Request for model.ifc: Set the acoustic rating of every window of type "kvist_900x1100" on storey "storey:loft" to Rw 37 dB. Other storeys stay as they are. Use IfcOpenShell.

First a look at what the model holds.

```python
import ifcopenshell
import ifcopenshell.util.element

model = ifcopenshell.open("model.ifc")
print(model.schema)
storey = next(s for s in model.by_type("IfcBuildingStorey") if s.Name == "storey:loft")
windows = [e for e in ifcopenshell.util.element.get_decomposition(storey) if e.is_a("IfcWindow")]
seen = {}
for e in windows:
    element_type = ifcopenshell.util.element.get_type(e)
    key = (element_type.Name if element_type != e and element_type else None, ifcopenshell.util.element.get_pset(e, "Pset_WindowCommon", "AcousticRating"))
    seen[key] = seen.get(key, 0) + 1
for (name, value), count in sorted(seen.items(), key=str):
    print(count, "x", name, "|", value)
```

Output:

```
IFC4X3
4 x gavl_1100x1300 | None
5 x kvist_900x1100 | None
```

```python
import ifcopenshell
import ifcopenshell.api.pset
import ifcopenshell.util.element

model = ifcopenshell.open("model.ifc")

storey = next(s for s in model.by_type("IfcBuildingStorey") if s.Name == "storey:loft")
windows = [e for e in ifcopenshell.util.element.get_decomposition(storey) if e.is_a("IfcWindow")]

count = 0
for e in windows:
    element_type = ifcopenshell.util.element.get_type(e)
    if element_type in (None, e) or element_type.Name != "kvist_900x1100":
        continue
    # add_pset returns the element's existing set when there is one.
    pset = ifcopenshell.api.pset.add_pset(model, product=e, name="Pset_WindowCommon")
    ifcopenshell.api.pset.edit_pset(model, pset=pset, properties={"AcousticRating": "Rw 37 dB"})
    count += 1

print(count, "windows updated")

model.write("model-out.ifc")
```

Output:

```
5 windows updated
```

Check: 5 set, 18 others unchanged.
